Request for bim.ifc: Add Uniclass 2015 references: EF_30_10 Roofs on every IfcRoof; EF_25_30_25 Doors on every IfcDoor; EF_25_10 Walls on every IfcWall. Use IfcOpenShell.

First a look at what the model holds.

```python
import ifcopenshell

model = ifcopenshell.open("bim.ifc")
print(model.schema)
print("classifications:", [c.Name for c in model.by_type("IfcClassification")])
for ifc_class in ("IfcDoor", "IfcRoof", "IfcStair", "IfcWall", "IfcWindow"):
    print(ifc_class, len(model.by_type(ifc_class)))
```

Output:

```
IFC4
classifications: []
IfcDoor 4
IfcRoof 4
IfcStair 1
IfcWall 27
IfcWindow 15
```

```python
import ifcopenshell
import ifcopenshell.api.classification

model = ifcopenshell.open("bim.ifc")

system = ifcopenshell.api.classification.add_classification(model, classification="Uniclass 2015")

codes = {
    "IfcRoof": ("EF_30_10", "Roofs"),
    "IfcDoor": ("EF_25_30_25", "Doors"),
    "IfcWall": ("EF_25_10", "Walls"),
}
for ifc_class, (code, name) in codes.items():
    products = model.by_type(ifc_class)
    ifcopenshell.api.classification.add_reference(
        model, products=products, classification=system, identification=code, name=name
    )
    print(code, len(products))

model.write("bim_updated.ifc")
```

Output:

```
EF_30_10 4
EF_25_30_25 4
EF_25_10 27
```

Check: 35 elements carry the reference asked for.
